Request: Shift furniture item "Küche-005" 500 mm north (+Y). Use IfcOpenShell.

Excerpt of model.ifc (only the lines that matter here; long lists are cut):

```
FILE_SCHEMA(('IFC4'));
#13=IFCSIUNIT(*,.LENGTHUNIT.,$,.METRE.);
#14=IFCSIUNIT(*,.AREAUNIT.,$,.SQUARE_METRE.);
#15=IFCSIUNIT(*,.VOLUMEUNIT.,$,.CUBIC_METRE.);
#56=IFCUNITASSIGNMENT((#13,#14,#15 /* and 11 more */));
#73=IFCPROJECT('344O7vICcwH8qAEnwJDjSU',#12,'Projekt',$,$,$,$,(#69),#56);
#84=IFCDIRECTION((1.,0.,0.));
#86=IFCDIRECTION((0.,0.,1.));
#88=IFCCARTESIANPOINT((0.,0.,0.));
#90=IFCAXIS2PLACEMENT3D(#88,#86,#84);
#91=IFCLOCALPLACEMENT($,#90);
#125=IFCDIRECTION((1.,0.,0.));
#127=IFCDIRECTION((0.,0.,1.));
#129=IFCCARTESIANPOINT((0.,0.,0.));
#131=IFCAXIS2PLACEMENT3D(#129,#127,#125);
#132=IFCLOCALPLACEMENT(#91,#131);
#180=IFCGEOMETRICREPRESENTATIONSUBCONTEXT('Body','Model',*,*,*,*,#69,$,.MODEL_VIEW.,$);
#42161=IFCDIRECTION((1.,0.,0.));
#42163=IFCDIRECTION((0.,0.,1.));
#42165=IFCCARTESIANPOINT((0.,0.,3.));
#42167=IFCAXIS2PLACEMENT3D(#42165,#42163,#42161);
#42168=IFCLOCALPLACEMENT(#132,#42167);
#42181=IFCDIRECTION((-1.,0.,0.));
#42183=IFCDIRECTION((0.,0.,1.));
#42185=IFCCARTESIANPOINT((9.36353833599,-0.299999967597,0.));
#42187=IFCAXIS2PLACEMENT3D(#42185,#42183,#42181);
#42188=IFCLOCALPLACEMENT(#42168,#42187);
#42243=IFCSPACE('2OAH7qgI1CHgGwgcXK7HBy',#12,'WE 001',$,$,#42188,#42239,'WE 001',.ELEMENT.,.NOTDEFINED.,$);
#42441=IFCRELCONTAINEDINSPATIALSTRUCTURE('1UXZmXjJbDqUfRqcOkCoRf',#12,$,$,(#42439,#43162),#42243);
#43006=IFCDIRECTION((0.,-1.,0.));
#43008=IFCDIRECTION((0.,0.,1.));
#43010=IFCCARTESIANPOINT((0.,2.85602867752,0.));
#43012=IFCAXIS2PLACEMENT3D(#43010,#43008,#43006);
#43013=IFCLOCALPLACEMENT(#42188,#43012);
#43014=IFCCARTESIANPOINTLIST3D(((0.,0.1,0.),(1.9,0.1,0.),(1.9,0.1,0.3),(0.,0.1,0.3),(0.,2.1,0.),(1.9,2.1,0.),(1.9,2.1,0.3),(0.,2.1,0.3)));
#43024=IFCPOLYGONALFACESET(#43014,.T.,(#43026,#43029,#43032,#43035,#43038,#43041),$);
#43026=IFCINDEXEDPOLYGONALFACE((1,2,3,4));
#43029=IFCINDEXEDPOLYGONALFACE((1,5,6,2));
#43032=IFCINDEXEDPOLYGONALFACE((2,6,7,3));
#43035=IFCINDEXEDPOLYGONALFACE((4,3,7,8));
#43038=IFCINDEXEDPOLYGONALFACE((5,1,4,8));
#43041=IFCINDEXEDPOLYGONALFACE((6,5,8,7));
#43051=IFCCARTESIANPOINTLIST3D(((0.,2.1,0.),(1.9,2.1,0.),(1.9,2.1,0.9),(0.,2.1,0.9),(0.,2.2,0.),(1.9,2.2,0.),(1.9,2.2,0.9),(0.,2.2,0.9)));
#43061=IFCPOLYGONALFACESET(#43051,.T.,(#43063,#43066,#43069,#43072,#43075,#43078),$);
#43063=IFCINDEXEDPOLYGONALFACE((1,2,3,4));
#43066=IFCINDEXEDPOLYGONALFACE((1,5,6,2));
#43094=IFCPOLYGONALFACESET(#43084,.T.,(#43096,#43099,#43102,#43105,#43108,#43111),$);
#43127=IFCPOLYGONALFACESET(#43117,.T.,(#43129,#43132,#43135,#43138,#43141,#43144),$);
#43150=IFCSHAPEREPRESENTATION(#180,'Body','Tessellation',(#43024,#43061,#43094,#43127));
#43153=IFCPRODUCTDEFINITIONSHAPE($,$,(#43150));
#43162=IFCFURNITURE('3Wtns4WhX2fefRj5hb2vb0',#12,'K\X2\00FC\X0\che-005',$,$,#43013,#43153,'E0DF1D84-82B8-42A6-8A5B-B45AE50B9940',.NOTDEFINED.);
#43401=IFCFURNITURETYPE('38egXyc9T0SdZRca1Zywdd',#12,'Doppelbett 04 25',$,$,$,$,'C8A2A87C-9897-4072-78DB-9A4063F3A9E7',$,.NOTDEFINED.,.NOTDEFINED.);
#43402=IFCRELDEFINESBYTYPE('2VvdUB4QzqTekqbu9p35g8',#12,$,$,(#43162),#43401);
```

```python
import ifcopenshell
import ifcopenshell.api.geometry
import ifcopenshell.util.placement
import ifcopenshell.util.unit

model = ifcopenshell.open("model.ifc")
unit_scale = ifcopenshell.util.unit.calculate_unit_scale(model)

item = model.by_id(43162)
matrix = ifcopenshell.util.placement.get_local_placement(item.ObjectPlacement)
matrix[1, 3] += 0.5 / unit_scale
ifcopenshell.api.geometry.edit_object_placement(model, product=item, matrix=matrix, is_si=False)

print(ifcopenshell.util.placement.get_local_placement(item.ObjectPlacement).round(3) + 0.0)

model.write("model_updated.ifc")
```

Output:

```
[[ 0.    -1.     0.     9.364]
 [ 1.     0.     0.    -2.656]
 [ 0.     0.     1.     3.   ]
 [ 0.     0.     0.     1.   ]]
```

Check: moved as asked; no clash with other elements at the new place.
